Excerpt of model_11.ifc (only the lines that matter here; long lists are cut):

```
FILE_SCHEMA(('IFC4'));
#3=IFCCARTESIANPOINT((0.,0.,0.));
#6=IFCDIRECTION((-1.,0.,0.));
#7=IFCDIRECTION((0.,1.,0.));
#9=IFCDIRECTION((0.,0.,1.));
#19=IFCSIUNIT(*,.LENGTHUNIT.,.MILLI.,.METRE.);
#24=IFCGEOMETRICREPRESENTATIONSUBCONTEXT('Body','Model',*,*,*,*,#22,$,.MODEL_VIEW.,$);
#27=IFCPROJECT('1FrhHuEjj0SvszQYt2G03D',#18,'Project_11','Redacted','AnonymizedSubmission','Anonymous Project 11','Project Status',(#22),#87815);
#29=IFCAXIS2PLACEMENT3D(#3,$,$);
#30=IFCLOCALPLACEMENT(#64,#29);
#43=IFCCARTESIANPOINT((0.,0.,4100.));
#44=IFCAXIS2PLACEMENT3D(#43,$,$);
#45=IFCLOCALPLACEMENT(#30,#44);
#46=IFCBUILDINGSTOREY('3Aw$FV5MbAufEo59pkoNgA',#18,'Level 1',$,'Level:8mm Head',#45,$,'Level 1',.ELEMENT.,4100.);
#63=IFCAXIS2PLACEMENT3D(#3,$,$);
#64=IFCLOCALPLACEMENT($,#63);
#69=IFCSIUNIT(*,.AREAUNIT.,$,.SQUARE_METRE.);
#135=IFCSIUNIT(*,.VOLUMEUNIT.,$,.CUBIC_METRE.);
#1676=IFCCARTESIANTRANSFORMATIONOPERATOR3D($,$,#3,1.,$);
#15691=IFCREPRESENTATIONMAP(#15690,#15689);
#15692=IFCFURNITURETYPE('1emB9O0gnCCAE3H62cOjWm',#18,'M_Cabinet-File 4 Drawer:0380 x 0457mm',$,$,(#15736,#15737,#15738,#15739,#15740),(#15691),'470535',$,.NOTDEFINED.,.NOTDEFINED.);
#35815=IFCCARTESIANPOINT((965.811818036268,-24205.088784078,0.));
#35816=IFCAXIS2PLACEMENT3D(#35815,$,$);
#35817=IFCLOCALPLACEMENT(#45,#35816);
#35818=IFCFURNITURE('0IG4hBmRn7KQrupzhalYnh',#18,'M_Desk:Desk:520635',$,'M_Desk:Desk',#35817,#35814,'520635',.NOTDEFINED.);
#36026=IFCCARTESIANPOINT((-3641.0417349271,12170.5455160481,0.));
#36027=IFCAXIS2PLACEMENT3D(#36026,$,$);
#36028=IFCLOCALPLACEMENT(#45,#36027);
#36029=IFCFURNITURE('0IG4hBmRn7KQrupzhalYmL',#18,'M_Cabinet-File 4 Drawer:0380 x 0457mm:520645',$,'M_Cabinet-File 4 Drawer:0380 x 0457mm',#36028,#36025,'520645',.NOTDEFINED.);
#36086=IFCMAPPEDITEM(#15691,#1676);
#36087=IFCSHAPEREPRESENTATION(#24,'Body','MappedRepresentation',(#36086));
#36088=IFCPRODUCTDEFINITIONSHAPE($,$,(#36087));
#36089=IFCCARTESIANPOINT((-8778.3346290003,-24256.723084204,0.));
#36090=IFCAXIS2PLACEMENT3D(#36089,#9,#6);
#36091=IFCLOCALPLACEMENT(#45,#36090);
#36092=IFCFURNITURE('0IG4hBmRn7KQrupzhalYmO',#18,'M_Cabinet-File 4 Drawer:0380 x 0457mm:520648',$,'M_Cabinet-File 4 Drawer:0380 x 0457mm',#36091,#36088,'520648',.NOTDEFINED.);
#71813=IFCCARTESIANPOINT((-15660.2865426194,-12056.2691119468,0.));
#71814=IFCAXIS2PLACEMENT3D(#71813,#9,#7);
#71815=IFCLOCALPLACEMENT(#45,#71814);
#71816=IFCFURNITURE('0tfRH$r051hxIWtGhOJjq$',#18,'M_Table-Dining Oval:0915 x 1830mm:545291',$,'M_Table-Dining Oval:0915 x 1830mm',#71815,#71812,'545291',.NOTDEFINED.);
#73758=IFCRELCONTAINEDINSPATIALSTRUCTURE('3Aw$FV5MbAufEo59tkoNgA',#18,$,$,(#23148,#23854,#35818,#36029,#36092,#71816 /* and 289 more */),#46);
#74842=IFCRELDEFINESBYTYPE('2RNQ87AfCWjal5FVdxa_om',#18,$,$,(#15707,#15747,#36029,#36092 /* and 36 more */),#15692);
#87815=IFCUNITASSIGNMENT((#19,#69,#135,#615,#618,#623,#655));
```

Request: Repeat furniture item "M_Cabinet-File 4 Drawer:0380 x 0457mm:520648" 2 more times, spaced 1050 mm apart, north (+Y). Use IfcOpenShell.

```python
import numpy as np
import ifcopenshell
import ifcopenshell.api.geometry
import ifcopenshell.api.root
import ifcopenshell.util.element
import ifcopenshell.util.placement

model = ifcopenshell.open("model_11.ifc")


def reuse_history(source, copy):
    """copy_class also copies each property set's owner history, people and application; keep the originals."""
    for rel in copy.IsDefinedBy:
        if rel.is_a("IfcRelDefinesByProperties") and (history := rel.RelatingPropertyDefinition.OwnerHistory):
            rel.RelatingPropertyDefinition.OwnerHistory = source.OwnerHistory
            ifcopenshell.util.element.remove_deep2(model, history)


source = model.by_id(36092)
base = ifcopenshell.util.placement.get_local_placement(source.ObjectPlacement)
step = np.array([0.0, 1.0, 0.0]) * 1050.0

for i in range(1, 3):
    copy = ifcopenshell.api.root.copy_class(model, product=source)
    copy.Representation = ifcopenshell.util.element.copy_deep(
        model, source.Representation, exclude=["IfcGeometricRepresentationContext", "IfcRepresentationMap"]
    )
    copy.Name = "M_Cabinet-File 4 Drawer:0380 x 0457mm"
    copy.Tag = None
    reuse_history(source, copy)
    matrix = base.copy()
    matrix[:3, 3] += i * step
    print("added at", matrix[:3, 3].round(3) + 0.0)
    ifcopenshell.api.geometry.edit_object_placement(model, product=copy, matrix=matrix, is_si=False)

model.write("model_11_v2.ifc")
```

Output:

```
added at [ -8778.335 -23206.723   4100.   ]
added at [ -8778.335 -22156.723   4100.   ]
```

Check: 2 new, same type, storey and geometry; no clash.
